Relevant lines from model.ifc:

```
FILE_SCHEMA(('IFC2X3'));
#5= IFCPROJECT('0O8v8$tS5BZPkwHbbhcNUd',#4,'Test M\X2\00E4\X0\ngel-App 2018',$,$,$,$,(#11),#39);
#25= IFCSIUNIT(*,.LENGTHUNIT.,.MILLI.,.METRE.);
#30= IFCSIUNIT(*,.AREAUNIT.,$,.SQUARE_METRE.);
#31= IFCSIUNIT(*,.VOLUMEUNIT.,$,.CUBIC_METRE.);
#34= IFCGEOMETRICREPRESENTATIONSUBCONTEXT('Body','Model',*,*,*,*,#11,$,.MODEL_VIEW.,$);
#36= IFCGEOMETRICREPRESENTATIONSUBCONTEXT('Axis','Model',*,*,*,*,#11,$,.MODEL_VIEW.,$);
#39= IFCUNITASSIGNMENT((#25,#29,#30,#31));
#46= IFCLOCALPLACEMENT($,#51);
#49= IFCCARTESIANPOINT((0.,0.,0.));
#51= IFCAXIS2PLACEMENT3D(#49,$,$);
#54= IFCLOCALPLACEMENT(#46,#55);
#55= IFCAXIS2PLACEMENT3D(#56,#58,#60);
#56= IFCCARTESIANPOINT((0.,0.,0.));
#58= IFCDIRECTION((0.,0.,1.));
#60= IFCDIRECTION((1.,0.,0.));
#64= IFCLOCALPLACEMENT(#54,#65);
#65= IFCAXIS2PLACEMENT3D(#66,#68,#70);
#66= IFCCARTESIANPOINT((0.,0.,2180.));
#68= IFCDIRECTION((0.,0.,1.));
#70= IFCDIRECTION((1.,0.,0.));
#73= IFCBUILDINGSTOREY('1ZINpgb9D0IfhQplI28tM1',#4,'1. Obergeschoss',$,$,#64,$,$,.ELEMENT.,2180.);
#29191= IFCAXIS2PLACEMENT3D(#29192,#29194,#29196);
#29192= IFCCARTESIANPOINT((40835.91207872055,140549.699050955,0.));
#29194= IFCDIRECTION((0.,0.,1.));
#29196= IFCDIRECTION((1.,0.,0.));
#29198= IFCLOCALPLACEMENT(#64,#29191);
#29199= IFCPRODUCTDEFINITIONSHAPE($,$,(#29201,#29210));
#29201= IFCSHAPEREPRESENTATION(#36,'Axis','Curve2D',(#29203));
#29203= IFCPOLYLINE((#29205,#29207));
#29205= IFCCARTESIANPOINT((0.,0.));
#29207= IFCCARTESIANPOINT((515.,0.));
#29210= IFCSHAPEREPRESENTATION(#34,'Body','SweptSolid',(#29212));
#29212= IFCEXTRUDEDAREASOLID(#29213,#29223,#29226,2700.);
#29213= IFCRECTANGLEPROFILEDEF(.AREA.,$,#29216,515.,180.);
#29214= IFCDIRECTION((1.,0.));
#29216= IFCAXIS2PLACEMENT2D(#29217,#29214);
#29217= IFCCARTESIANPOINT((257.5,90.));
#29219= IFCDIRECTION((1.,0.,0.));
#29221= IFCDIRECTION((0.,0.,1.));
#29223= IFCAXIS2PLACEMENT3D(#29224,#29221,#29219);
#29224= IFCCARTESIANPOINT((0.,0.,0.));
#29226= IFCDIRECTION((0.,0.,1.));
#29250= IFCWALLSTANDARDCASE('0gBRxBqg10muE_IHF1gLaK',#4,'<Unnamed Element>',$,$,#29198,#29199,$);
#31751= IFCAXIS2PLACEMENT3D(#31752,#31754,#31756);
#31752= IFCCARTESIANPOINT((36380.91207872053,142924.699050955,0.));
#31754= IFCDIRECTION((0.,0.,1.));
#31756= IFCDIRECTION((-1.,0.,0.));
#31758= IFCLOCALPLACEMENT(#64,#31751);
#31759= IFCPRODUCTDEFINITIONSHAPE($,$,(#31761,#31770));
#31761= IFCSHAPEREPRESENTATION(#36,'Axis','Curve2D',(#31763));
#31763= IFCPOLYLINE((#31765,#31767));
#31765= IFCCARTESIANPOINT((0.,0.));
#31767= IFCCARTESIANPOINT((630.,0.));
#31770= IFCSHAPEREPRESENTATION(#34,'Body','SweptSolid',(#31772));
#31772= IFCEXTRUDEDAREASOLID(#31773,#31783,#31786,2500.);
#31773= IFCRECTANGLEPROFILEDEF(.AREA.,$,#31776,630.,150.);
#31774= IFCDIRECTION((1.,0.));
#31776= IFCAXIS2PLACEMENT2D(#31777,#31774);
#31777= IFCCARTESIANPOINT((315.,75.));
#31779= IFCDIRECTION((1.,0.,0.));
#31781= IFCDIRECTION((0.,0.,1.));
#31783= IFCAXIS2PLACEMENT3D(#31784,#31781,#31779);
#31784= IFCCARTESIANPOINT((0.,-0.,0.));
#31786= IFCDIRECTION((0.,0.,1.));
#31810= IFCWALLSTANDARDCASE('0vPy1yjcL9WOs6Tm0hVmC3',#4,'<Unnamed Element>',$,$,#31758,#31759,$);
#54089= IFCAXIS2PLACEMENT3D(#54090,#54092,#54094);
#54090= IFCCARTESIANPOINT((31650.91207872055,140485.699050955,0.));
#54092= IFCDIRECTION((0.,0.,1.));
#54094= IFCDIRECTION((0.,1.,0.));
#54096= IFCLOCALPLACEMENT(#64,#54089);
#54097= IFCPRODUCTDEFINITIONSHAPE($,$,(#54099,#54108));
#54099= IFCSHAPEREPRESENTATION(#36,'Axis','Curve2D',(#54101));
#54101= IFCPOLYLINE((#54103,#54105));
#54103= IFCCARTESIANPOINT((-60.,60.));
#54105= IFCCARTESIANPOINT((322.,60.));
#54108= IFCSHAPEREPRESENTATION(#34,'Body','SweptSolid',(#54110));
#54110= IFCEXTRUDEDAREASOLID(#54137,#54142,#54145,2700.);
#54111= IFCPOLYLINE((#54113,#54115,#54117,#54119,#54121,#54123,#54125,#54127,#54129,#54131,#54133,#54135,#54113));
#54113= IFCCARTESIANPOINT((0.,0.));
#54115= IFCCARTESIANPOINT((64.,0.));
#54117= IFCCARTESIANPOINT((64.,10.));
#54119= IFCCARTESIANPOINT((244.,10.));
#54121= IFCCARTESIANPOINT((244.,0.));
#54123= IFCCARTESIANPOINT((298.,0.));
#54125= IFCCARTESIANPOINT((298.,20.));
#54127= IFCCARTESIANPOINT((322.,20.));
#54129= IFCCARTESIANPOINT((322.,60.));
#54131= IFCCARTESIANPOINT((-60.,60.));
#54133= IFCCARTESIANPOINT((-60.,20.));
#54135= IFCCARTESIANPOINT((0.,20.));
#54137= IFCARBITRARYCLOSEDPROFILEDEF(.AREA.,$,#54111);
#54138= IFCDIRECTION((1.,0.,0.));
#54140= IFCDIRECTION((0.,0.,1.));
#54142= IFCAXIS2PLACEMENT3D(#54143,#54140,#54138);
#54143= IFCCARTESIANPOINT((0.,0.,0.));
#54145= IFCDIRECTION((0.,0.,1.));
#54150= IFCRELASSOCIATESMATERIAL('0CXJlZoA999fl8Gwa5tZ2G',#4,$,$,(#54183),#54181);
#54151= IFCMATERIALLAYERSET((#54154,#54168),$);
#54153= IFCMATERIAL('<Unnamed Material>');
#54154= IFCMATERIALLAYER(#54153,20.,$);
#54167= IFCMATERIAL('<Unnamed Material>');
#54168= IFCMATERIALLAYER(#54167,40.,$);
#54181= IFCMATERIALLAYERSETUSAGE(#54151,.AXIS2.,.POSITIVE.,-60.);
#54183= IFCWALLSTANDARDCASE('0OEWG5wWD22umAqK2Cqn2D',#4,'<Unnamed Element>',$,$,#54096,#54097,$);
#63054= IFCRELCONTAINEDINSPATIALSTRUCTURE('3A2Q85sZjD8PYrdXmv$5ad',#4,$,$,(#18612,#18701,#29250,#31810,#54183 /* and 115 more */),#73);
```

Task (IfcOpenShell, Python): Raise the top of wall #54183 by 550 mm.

```python
import ifcopenshell
import ifcopenshell.geom
import ifcopenshell.util.representation
import ifcopenshell.util.shape
import ifcopenshell.util.unit

model = ifcopenshell.open("model.ifc")
unit_scale = ifcopenshell.util.unit.calculate_unit_scale(model)
settings = ifcopenshell.geom.settings()


def volume(element):
    """Net volume in cubic metres, openings subtracted."""
    shape = ifcopenshell.geom.create_shape(settings, element)
    return ifcopenshell.util.shape.get_volume(shape.geometry)


wall = model.by_id(54183)
before = volume(wall)

body = ifcopenshell.util.representation.get_representation(wall, "Model", "Body")
solid = body.Items[0]
old_height = solid.Depth
solid.Depth += 0.55 / unit_scale
after = volume(wall)

print(f"height {old_height:g} -> {solid.Depth:g}, volume {before:.3f} -> {after:.3f} m3")

model.write("model_rev.ifc")
```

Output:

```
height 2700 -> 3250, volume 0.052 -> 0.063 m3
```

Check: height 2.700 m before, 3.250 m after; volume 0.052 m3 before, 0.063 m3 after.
